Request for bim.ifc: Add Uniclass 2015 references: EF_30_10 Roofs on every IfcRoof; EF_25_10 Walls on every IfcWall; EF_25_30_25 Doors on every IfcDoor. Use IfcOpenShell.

First a look at what the model holds.

```python
import ifcopenshell

model = ifcopenshell.open("bim.ifc")
print(model.schema)
print("classifications:", [c.Name for c in model.by_type("IfcClassification")])
for ifc_class in ("IfcDoor", "IfcRoof", "IfcStair", "IfcWall", "IfcWindow"):
    print(ifc_class, len(model.by_type(ifc_class)))
```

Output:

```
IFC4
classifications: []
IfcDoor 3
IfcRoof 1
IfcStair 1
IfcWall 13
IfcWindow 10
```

```python
import ifcopenshell
import ifcopenshell.api.classification

model = ifcopenshell.open("bim.ifc")

system = ifcopenshell.api.classification.add_classification(model, classification="Uniclass 2015")

codes = {
    "IfcRoof": ("EF_30_10", "Roofs"),
    "IfcWall": ("EF_25_10", "Walls"),
    "IfcDoor": ("EF_25_30_25", "Doors"),
}
for ifc_class, (code, name) in codes.items():
    products = model.by_type(ifc_class)
    ifcopenshell.api.classification.add_reference(
        model, products=products, classification=system, identification=code, name=name
    )
    print(code, len(products))

model.write("bim_updated.ifc")
```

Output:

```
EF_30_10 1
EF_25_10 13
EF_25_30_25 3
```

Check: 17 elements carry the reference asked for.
